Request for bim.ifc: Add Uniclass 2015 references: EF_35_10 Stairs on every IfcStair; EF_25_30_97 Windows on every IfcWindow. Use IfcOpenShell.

First a look at what the model holds.

```python
import ifcopenshell

model = ifcopenshell.open("bim.ifc")
print(model.schema)
print("classifications:", [c.Name for c in model.by_type("IfcClassification")])
for ifc_class in ("IfcDoor", "IfcRoof", "IfcStair", "IfcWall", "IfcWindow"):
    print(ifc_class, len(model.by_type(ifc_class)))
```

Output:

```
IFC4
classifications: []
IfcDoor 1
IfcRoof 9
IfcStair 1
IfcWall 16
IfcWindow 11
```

```python
import ifcopenshell
import ifcopenshell.api.classification

model = ifcopenshell.open("bim.ifc")

system = ifcopenshell.api.classification.add_classification(model, classification="Uniclass 2015")

codes = {
    "IfcStair": ("EF_35_10", "Stairs"),
    "IfcWindow": ("EF_25_30_97", "Windows"),
}
for ifc_class, (code, name) in codes.items():
    products = model.by_type(ifc_class)
    ifcopenshell.api.classification.add_reference(
        model, products=products, classification=system, identification=code, name=name
    )
    print(code, len(products))

model.write("bim_updated.ifc")
```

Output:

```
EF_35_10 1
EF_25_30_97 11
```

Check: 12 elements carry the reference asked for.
